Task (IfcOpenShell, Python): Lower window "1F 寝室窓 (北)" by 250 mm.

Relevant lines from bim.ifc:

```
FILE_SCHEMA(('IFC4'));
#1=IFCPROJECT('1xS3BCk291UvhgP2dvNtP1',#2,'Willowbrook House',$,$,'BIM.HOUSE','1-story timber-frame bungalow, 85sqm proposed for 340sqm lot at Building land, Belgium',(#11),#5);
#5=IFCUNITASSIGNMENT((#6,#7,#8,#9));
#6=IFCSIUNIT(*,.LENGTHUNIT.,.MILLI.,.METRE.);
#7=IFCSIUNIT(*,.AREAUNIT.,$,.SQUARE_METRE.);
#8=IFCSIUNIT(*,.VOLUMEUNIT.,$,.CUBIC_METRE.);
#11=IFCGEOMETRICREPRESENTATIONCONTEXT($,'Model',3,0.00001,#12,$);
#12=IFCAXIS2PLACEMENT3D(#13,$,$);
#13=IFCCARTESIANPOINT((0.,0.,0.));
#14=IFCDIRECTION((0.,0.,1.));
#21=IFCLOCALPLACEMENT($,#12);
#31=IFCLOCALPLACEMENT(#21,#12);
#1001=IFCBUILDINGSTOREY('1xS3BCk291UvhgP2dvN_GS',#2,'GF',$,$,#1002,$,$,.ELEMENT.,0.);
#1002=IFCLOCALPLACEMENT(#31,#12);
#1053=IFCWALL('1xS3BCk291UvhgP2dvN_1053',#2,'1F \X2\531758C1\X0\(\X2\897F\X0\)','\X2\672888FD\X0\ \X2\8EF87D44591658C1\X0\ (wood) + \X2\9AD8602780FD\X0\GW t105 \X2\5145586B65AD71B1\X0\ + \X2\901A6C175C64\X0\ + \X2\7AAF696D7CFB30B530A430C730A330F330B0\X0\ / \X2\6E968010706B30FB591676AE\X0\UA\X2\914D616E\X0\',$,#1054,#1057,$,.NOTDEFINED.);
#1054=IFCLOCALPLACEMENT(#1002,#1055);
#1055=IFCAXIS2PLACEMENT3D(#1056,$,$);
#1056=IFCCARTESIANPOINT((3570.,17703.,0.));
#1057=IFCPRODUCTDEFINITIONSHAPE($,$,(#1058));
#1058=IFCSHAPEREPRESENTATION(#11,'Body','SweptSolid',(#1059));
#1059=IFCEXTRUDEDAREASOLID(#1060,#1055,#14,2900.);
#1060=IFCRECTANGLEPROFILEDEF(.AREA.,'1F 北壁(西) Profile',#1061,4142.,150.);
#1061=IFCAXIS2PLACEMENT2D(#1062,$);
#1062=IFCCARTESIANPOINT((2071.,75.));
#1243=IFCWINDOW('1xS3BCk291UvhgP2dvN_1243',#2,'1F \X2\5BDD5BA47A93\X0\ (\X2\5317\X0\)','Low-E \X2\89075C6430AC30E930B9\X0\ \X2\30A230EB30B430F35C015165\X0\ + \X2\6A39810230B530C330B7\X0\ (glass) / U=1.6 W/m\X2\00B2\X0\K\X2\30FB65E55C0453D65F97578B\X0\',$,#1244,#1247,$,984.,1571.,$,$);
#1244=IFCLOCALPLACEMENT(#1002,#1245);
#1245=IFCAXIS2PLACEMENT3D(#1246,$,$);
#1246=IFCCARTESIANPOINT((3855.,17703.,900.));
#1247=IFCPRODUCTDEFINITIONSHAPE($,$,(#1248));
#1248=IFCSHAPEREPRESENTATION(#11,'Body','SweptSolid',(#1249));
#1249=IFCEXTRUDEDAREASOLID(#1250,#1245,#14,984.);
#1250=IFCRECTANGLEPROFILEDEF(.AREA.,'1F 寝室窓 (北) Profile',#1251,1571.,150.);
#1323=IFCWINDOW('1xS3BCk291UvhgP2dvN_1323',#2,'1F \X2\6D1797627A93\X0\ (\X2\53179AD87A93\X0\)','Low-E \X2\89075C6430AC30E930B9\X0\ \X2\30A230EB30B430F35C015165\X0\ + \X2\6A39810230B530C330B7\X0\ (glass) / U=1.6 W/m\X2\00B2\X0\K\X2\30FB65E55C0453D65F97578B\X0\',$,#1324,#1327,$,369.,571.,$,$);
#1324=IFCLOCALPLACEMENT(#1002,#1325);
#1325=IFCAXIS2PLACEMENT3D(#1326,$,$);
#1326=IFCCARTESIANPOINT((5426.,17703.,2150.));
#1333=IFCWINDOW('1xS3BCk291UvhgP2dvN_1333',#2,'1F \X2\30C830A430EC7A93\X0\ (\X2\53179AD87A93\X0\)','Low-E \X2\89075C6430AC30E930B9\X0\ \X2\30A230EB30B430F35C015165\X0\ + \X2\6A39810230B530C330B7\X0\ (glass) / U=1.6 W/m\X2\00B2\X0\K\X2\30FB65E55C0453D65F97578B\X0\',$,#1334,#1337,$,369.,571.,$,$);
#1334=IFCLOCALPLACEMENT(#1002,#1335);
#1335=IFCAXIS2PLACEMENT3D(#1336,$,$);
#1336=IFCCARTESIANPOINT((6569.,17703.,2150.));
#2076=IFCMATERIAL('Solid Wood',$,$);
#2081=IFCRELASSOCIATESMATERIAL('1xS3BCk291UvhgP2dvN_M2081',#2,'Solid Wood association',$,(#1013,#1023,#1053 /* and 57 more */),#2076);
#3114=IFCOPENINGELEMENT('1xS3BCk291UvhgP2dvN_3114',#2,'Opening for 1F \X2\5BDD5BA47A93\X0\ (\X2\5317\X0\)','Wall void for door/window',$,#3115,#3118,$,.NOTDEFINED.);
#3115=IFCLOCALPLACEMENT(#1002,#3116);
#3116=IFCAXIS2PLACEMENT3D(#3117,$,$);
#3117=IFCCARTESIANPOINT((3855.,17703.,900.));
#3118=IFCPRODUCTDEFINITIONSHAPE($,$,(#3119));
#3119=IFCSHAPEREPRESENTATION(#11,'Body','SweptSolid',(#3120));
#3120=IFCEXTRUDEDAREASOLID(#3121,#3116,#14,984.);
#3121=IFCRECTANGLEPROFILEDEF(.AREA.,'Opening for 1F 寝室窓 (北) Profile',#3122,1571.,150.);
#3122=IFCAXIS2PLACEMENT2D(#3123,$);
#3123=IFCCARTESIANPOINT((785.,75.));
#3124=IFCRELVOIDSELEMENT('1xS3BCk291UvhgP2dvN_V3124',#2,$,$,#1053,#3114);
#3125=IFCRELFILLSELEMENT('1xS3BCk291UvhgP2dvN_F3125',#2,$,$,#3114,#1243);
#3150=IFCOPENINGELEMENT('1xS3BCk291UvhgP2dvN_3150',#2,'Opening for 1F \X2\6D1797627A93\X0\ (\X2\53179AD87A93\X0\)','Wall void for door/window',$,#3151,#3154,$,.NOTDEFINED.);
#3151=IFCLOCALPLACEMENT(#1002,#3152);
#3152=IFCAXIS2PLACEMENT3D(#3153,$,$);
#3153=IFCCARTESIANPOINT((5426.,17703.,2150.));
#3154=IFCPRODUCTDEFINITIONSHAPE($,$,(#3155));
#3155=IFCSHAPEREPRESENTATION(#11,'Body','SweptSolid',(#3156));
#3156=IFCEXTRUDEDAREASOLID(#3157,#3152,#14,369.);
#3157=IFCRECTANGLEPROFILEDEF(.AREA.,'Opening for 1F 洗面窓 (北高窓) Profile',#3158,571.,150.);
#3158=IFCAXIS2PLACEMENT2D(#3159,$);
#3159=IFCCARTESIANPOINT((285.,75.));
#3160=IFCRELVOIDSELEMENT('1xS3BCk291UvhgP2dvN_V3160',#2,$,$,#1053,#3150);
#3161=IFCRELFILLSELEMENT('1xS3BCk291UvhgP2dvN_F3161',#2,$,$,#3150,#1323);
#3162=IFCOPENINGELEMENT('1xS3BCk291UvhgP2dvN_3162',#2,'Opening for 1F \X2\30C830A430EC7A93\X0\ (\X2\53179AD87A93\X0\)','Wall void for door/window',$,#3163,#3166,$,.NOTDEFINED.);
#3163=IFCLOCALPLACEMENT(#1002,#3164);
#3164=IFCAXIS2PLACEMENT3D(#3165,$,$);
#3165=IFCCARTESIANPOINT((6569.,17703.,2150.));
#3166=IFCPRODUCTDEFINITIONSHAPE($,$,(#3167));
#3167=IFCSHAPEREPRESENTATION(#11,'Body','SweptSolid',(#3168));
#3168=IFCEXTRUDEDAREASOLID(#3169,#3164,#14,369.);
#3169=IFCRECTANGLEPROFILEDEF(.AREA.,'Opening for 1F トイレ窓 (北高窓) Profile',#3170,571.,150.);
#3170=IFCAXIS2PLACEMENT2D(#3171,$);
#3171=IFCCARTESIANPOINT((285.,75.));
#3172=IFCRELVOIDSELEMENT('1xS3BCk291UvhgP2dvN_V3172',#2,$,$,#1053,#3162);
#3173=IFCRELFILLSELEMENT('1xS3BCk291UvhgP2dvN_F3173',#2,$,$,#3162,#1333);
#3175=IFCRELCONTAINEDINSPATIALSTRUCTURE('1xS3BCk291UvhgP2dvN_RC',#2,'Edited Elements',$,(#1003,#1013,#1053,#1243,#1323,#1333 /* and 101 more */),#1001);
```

```python
import numpy as np
import ifcopenshell
import ifcopenshell.api.geometry
import ifcopenshell.util.placement
import ifcopenshell.util.unit

model = ifcopenshell.open("bim.ifc")
unit_scale = ifcopenshell.util.unit.calculate_unit_scale(model)

window = model.by_guid("1xS3BCk291UvhgP2dvN_1243")
opening = window.FillsVoids[0].RelatingOpeningElement
dz = -0.25 / unit_scale

shift = np.array([0.0, 0.0, dz])
# The window is not placed relative to its opening, so move both.
for product in (opening, window):
    matrix = ifcopenshell.util.placement.get_local_placement(product.ObjectPlacement)
    matrix[:3, 3] += shift
    ifcopenshell.api.geometry.edit_object_placement(model, product=product, matrix=matrix, is_si=False)

print(f"moved by {dz * unit_scale:+.3f} m")

model.write("bim_rev.ifc")
```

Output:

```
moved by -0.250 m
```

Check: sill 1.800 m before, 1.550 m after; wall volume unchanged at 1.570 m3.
